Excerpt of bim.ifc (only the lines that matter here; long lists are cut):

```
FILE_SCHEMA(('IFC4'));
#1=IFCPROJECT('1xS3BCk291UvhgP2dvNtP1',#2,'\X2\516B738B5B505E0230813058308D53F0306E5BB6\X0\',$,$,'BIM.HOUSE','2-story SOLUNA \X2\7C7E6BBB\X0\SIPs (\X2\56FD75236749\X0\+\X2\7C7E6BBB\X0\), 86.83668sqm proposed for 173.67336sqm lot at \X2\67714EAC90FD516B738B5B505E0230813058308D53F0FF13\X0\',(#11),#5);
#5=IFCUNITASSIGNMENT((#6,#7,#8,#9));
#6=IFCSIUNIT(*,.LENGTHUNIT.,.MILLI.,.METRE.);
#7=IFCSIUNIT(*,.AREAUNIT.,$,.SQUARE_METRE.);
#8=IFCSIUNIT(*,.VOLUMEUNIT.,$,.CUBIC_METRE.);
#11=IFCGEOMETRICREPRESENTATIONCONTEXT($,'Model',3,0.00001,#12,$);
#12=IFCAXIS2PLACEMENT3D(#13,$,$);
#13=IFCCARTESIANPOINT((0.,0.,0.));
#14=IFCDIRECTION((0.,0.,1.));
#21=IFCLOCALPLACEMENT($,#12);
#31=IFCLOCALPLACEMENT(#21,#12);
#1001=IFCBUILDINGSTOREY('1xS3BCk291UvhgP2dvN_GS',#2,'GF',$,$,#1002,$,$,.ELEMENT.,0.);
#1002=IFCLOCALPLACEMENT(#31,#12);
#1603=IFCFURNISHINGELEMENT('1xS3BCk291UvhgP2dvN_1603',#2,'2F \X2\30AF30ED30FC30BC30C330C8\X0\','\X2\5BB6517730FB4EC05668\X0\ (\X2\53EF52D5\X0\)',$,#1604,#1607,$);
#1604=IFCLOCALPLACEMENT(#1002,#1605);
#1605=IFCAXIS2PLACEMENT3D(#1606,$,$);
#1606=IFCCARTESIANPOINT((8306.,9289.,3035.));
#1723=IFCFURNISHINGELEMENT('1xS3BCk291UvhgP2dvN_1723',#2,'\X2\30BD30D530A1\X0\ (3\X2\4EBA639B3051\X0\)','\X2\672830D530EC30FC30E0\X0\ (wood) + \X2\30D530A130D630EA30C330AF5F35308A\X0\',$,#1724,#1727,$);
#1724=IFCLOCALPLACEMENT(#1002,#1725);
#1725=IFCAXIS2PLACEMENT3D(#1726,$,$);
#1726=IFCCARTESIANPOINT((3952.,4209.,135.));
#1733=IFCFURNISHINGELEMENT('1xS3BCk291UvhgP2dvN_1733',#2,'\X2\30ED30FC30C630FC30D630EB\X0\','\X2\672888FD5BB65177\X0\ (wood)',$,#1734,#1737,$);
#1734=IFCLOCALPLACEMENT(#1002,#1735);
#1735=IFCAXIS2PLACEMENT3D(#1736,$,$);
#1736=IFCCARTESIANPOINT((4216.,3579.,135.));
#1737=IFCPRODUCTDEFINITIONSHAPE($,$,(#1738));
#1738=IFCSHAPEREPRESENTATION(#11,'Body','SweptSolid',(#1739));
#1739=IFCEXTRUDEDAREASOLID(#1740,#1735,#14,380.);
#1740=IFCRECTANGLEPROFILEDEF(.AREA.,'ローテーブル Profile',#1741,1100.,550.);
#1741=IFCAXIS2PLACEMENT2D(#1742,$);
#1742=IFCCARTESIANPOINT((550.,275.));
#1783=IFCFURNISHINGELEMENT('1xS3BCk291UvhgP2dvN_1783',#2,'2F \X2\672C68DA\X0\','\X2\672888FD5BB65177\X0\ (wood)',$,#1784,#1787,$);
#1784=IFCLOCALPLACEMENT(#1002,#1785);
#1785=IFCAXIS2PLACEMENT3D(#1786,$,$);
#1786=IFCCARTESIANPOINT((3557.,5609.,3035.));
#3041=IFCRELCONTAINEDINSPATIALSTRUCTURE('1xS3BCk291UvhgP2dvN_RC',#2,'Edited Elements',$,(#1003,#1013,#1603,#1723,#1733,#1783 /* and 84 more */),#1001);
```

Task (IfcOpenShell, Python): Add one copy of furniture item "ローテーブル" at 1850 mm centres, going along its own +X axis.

```python
import ifcopenshell
import ifcopenshell.api.geometry
import ifcopenshell.api.root
import ifcopenshell.util.element
import ifcopenshell.util.placement
import ifcopenshell.util.unit

model = ifcopenshell.open("bim.ifc")
unit_scale = ifcopenshell.util.unit.calculate_unit_scale(model)


def reuse_history(source, copy):
    """copy_class also copies each property set's owner history, people and application; keep the originals."""
    for rel in copy.IsDefinedBy:
        if rel.is_a("IfcRelDefinesByProperties") and (history := rel.RelatingPropertyDefinition.OwnerHistory):
            rel.RelatingPropertyDefinition.OwnerHistory = source.OwnerHistory
            ifcopenshell.util.element.remove_deep2(model, history)


source = model.by_guid("1xS3BCk291UvhgP2dvN_1733")
base = ifcopenshell.util.placement.get_local_placement(source.ObjectPlacement)
step = base[:3, 0] * 1.85 / unit_scale

for i in range(1, 2):
    copy = ifcopenshell.api.root.copy_class(model, product=source)
    copy.Representation = ifcopenshell.util.element.copy_deep(
        model, source.Representation, exclude=["IfcGeometricRepresentationContext", "IfcRepresentationMap"]
    )
    reuse_history(source, copy)
    matrix = base.copy()
    matrix[:3, 3] += i * step
    print("added at", matrix[:3, 3].round(3) + 0.0)
    ifcopenshell.api.geometry.edit_object_placement(model, product=copy, matrix=matrix, is_si=False)

model.write("bim_updated.ifc")
```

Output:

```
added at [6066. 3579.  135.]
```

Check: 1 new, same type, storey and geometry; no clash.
